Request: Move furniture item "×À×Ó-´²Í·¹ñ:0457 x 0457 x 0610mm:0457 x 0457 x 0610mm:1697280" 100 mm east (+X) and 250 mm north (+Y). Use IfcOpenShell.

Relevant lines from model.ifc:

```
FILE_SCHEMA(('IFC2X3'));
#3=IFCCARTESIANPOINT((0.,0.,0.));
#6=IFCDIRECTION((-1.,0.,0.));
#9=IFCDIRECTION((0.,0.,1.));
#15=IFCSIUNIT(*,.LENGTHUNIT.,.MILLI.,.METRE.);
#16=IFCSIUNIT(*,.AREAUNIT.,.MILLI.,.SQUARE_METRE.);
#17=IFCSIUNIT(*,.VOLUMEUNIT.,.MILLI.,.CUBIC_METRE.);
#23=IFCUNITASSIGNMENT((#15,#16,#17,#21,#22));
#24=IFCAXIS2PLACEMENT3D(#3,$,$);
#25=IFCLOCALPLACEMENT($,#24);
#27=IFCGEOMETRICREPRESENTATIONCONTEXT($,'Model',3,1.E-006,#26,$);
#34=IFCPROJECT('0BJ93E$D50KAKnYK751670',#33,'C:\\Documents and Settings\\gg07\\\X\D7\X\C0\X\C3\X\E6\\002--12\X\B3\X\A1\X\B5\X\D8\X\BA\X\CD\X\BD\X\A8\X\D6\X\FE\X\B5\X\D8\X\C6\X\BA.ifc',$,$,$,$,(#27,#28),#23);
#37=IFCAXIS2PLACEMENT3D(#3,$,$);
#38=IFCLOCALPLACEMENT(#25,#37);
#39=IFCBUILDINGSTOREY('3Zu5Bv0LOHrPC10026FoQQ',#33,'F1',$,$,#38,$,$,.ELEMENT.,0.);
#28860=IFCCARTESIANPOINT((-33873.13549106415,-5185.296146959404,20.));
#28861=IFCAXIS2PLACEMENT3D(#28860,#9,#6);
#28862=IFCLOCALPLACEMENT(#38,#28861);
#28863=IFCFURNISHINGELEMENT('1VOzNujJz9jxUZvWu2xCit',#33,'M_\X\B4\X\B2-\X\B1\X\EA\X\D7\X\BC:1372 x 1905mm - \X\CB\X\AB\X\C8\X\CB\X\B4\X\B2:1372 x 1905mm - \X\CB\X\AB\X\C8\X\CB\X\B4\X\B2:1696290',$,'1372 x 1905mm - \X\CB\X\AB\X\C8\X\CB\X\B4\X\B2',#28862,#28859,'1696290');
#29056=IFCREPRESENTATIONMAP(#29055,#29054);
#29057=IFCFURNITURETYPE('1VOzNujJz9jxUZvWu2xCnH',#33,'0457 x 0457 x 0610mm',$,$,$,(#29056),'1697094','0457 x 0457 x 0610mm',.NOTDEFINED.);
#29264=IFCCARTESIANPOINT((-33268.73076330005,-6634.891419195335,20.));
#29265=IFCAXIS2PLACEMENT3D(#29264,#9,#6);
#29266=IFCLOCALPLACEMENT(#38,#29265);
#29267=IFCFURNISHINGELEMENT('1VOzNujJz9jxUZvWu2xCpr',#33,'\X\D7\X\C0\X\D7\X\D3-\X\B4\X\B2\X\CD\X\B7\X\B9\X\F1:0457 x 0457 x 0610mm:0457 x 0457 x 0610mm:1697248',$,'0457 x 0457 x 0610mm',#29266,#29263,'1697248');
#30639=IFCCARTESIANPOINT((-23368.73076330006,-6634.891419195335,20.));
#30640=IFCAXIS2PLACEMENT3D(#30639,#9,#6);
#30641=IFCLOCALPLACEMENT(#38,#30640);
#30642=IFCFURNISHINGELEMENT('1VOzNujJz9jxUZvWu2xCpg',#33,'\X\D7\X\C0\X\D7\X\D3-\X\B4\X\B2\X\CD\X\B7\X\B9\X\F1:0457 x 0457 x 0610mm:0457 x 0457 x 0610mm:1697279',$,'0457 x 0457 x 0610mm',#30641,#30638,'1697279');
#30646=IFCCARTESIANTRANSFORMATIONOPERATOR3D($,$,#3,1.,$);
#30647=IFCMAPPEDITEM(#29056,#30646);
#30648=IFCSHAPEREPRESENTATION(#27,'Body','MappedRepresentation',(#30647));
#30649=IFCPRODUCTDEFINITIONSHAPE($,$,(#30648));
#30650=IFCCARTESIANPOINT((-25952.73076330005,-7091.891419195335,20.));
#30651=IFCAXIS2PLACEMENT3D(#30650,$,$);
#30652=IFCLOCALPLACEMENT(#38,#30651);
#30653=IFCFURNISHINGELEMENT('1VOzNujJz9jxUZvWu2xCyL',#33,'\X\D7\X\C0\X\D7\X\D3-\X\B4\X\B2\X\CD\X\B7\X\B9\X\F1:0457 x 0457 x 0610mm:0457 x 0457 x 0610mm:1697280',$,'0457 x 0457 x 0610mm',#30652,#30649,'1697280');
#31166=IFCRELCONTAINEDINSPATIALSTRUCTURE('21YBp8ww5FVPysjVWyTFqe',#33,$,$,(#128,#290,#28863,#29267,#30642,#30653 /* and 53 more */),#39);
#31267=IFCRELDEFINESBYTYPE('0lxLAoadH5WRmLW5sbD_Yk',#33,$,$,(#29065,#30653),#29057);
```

```python
import ifcopenshell
import ifcopenshell.api.geometry
import ifcopenshell.util.placement
import ifcopenshell.util.unit

model = ifcopenshell.open("model.ifc")
unit_scale = ifcopenshell.util.unit.calculate_unit_scale(model)

item = model.by_guid("1VOzNujJz9jxUZvWu2xCyL")
matrix = ifcopenshell.util.placement.get_local_placement(item.ObjectPlacement)
matrix[0, 3] += 0.1 / unit_scale
matrix[1, 3] += 0.25 / unit_scale
ifcopenshell.api.geometry.edit_object_placement(model, product=item, matrix=matrix, is_si=False)

print(ifcopenshell.util.placement.get_local_placement(item.ObjectPlacement).round(3) + 0.0)

model.write("model_edited.ifc")
```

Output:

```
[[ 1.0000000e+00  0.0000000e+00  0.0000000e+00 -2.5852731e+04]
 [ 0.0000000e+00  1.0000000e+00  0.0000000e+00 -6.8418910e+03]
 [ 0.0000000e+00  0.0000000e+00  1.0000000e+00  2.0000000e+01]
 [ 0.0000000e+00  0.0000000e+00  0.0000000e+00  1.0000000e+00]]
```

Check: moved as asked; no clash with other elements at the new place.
